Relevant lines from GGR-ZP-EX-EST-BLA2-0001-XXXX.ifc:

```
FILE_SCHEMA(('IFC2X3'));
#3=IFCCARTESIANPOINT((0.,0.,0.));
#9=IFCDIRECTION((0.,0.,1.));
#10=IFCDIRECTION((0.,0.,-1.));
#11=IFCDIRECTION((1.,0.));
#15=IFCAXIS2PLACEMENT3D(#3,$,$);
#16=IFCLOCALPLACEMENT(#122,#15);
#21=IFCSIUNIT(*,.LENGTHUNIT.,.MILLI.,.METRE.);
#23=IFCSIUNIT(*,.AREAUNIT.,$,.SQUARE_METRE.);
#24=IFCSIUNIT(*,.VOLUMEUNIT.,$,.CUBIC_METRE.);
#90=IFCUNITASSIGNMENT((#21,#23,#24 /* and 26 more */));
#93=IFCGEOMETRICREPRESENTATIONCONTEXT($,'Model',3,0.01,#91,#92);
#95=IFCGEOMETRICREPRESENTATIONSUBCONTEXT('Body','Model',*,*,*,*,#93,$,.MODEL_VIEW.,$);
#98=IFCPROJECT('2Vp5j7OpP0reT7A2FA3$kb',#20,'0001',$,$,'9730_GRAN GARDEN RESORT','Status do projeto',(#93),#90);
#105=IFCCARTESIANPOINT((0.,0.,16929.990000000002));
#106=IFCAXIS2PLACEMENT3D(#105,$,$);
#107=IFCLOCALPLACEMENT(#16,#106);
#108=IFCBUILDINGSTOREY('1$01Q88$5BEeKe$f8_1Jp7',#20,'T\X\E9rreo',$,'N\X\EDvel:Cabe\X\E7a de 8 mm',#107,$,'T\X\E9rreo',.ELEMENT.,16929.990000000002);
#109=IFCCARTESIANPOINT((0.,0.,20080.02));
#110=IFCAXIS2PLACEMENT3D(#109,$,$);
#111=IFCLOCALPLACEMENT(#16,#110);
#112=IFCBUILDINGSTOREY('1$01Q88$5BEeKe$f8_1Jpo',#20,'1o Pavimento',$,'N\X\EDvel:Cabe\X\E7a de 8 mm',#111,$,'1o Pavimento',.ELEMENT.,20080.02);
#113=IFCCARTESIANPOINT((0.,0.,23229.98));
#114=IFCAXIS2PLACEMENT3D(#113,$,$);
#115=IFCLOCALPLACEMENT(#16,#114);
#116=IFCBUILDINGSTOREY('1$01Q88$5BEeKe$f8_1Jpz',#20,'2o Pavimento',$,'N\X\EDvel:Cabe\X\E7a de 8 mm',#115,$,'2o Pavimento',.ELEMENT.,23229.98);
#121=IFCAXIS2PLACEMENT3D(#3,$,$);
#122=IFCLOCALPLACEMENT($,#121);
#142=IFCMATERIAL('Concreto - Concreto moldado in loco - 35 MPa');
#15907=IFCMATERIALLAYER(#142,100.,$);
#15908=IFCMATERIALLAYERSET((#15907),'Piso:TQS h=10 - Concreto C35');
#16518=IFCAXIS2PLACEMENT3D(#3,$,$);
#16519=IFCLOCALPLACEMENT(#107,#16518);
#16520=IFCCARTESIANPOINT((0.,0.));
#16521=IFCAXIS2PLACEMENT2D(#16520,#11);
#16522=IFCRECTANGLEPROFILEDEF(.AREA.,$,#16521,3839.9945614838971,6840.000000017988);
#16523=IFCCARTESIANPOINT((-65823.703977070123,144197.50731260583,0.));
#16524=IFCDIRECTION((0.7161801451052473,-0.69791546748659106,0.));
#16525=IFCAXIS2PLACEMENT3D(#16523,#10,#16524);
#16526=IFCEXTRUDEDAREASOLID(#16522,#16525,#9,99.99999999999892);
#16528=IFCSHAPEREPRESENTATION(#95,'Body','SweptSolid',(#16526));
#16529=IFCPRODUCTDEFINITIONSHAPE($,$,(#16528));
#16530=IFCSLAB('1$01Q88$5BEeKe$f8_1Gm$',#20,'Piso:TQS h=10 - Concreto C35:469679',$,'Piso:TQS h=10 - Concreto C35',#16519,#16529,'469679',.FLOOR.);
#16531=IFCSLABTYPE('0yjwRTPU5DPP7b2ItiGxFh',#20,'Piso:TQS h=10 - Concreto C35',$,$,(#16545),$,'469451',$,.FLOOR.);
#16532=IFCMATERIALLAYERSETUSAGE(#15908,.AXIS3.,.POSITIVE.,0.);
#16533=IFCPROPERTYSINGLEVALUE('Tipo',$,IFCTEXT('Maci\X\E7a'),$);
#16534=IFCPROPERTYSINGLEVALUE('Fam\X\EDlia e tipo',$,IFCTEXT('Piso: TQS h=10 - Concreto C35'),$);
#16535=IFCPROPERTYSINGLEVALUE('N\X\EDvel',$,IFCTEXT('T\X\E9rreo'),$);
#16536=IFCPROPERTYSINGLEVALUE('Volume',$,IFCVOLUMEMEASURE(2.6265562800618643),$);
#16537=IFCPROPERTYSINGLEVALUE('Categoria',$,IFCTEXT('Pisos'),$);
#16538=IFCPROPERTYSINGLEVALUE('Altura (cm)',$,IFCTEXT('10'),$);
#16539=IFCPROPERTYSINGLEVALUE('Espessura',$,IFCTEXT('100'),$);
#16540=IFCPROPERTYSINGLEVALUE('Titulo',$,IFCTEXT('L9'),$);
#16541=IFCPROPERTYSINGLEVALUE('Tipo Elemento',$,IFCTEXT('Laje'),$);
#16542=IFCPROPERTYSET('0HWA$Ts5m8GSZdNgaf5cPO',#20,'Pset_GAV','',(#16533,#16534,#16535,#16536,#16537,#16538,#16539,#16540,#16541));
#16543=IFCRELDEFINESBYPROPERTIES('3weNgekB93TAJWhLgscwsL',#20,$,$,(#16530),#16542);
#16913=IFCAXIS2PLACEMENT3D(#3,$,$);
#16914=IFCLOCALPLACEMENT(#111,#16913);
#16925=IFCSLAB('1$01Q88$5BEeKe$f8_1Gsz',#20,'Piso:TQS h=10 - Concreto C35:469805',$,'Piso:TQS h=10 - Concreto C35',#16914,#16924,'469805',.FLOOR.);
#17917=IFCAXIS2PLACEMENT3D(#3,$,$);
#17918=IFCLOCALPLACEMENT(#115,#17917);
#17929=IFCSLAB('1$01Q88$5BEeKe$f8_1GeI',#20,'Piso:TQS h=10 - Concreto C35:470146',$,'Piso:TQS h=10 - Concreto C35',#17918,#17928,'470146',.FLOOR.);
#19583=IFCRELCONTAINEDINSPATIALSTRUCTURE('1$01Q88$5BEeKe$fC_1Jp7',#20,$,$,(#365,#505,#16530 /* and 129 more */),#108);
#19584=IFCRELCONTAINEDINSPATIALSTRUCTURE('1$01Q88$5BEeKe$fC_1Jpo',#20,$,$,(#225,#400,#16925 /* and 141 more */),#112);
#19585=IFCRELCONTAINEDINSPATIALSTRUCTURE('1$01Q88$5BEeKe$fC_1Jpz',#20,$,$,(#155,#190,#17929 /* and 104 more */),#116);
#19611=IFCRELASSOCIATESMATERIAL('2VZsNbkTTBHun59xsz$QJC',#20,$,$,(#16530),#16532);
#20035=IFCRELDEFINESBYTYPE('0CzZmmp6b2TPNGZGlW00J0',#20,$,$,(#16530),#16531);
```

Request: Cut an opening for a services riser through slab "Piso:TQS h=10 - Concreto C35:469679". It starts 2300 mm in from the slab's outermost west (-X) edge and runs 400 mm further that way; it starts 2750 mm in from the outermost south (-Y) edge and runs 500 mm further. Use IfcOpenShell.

```python
import numpy as np
import ifcopenshell
import ifcopenshell.api.feature
import ifcopenshell.api.geometry
import ifcopenshell.api.pset
import ifcopenshell.api.root
import ifcopenshell.geom
import ifcopenshell.util.element
import ifcopenshell.util.placement
import ifcopenshell.util.representation
import ifcopenshell.util.shape
import ifcopenshell.util.unit

model = ifcopenshell.open("GGR-ZP-EX-EST-BLA2-0001-XXXX.ifc")
unit_scale = ifcopenshell.util.unit.calculate_unit_scale(model)
volume_scale = ifcopenshell.util.unit.calculate_unit_scale(model, "VOLUMEUNIT")
settings = ifcopenshell.geom.settings()


def volume(element):
    """Net volume in cubic metres, openings subtracted."""
    shape = ifcopenshell.geom.create_shape(settings, element)
    return ifcopenshell.util.shape.get_volume(shape.geometry)


slab = model.by_guid("1$01Q88$5BEeKe$f8_1Gm$")
before = volume(slab)

# Extent in the slab's own axes, in metres. The edges named are its -X and -Y sides.
slab_shape = ifcopenshell.geom.create_shape(settings, slab)
vertices = ifcopenshell.util.shape.get_vertices(slab_shape.geometry)
x_min, y_min, bottom = vertices.min(axis=0)
top = vertices[:, 2].max()

opening = ifcopenshell.api.root.create_entity(model, ifc_class="IfcOpeningElement", name="Services riser opening")
context = ifcopenshell.util.representation.get_context(model, "Model", "Body", "MODEL_VIEW")
width, depth = 0.4, 0.5
outline = [(0.0, 0.0), (width, 0.0), (width, depth), (0.0, depth), (0.0, 0.0)]
# Overshoot both faces by 50 mm so the cut is clean.
shape = ifcopenshell.api.geometry.add_slab_representation(
    model, context=context, depth=top - bottom + 0.1, polyline=outline
)
ifcopenshell.api.geometry.assign_representation(model, product=opening, representation=shape)

matrix = ifcopenshell.util.placement.get_local_placement(slab.ObjectPlacement)
matrix[:, 3] = matrix @ np.append(np.array([x_min + 2.3, y_min + 2.75, bottom - 0.05]) / unit_scale, 1.0)
ifcopenshell.api.geometry.edit_object_placement(model, product=opening, matrix=matrix, is_si=False)
ifcopenshell.api.feature.add_feature(model, feature=opening, element=slab)

after = volume(slab)

# Update the slab's stored quantities.
pset = model.by_id(ifcopenshell.util.element.get_pset(slab, "Pset_GAV", should_inherit=False)["id"])
ifcopenshell.api.pset.edit_pset(model, pset=pset, properties={
    "Volume": model.create_entity("IfcVolumeMeasure", after / volume_scale),
})

print(f"slab volume {before:.3f} -> {after:.3f} m3")

model.write("GGR-ZP-EX-EST-BLA2-0001-XXXX_v2.ifc")
```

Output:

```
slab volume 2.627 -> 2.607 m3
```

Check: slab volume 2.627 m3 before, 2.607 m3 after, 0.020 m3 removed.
